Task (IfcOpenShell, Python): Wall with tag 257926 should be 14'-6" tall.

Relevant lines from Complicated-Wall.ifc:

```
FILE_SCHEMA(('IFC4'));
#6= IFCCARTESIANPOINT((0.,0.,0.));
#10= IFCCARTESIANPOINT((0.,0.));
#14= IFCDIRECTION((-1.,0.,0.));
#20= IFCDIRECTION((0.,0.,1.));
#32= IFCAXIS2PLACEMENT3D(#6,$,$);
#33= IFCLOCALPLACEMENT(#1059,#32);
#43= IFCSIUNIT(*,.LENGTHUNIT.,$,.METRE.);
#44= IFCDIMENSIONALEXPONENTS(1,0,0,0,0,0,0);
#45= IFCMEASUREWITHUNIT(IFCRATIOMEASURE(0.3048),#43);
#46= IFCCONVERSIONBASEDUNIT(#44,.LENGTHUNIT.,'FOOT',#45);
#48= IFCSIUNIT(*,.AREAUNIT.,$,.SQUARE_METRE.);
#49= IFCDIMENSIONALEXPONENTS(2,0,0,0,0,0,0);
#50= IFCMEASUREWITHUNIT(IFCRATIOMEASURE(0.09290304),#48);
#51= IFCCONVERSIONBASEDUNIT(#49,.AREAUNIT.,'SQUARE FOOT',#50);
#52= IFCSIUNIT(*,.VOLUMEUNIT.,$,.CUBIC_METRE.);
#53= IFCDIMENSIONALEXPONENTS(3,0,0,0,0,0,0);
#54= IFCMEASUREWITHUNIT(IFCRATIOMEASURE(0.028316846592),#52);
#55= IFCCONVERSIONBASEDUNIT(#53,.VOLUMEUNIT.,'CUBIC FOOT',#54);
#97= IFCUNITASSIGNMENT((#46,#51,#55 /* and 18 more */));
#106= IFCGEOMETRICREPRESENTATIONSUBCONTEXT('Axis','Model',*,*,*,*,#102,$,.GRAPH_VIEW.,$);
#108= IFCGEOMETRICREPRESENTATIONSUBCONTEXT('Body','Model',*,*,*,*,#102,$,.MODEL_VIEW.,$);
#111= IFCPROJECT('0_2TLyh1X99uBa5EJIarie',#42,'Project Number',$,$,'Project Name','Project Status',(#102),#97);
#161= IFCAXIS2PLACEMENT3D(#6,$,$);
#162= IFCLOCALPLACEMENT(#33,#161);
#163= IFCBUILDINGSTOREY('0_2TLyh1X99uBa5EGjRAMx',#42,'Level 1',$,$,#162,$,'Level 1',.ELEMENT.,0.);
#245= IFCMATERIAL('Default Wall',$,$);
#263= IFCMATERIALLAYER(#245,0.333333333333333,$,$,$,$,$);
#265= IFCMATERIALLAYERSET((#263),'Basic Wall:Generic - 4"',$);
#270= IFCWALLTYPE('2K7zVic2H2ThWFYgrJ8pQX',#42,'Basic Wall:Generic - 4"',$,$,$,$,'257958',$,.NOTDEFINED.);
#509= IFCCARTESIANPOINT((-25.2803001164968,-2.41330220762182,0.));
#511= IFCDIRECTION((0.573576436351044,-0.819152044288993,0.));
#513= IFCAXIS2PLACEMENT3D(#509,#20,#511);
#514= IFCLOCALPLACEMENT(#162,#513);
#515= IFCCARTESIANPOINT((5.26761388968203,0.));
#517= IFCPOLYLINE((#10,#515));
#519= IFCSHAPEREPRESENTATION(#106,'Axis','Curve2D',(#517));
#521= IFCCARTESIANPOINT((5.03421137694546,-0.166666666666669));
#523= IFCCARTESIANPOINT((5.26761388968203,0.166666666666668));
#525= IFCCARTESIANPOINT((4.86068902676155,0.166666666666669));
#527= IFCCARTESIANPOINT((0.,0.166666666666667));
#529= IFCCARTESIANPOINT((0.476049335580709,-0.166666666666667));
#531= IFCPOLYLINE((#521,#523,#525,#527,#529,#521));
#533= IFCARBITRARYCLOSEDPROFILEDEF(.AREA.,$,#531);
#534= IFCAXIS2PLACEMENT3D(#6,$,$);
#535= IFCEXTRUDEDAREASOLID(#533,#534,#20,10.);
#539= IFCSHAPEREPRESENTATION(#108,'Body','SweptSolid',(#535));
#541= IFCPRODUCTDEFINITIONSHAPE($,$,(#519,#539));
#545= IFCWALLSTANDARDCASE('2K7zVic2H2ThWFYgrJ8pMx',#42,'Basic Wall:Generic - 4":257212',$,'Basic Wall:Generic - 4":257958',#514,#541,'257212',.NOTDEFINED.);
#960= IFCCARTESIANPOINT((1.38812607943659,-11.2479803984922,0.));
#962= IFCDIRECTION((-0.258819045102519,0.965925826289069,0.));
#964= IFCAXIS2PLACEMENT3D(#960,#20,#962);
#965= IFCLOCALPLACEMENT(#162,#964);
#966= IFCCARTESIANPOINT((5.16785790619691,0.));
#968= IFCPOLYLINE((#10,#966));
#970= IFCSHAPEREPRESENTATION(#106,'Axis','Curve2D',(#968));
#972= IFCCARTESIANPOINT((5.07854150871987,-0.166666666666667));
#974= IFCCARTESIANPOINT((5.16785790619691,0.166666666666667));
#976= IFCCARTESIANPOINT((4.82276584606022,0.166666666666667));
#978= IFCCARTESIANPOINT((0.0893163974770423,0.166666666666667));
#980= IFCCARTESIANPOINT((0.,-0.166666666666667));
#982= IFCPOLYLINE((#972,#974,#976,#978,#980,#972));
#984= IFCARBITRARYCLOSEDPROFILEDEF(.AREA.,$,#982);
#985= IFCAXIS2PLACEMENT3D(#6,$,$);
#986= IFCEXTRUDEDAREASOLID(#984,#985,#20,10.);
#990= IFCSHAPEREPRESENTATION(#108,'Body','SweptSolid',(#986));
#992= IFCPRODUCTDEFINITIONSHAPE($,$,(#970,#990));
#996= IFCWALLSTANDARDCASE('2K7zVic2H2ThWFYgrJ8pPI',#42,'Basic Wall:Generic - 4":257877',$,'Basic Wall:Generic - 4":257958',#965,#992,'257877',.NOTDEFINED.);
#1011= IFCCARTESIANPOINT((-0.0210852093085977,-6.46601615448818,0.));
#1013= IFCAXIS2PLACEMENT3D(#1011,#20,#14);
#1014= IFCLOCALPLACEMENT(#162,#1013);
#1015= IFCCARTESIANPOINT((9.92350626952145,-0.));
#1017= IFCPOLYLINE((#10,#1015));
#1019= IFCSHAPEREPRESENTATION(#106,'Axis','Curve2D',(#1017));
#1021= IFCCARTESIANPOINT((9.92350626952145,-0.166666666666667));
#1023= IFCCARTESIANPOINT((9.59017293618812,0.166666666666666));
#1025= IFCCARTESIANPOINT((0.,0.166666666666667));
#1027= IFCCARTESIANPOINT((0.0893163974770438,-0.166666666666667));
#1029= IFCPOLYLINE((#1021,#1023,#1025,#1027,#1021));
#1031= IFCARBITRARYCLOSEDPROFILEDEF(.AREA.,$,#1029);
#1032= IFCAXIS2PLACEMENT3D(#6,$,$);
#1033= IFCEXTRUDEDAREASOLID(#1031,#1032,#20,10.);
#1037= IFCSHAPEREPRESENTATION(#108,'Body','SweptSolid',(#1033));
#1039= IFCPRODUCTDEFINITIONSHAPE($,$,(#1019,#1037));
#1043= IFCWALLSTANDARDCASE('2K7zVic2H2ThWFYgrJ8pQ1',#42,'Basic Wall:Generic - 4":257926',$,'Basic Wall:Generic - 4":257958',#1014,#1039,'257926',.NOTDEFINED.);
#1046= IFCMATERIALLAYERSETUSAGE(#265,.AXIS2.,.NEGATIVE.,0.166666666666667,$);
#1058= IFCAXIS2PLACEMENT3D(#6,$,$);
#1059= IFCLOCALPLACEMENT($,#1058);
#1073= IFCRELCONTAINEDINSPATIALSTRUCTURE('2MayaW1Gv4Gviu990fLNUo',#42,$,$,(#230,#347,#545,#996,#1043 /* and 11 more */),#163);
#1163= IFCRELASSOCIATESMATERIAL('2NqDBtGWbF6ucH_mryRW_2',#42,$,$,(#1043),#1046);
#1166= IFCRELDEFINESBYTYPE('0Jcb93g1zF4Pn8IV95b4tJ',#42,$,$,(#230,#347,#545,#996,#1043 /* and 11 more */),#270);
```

```python
import ifcopenshell
import ifcopenshell.geom
import ifcopenshell.util.representation
import ifcopenshell.util.shape
import ifcopenshell.util.unit

model = ifcopenshell.open("Complicated-Wall.ifc")
unit_scale = ifcopenshell.util.unit.calculate_unit_scale(model)
settings = ifcopenshell.geom.settings()


def volume(element):
    """Net volume in cubic metres, openings subtracted."""
    shape = ifcopenshell.geom.create_shape(settings, element)
    return ifcopenshell.util.shape.get_volume(shape.geometry)


wall = model.by_guid("2K7zVic2H2ThWFYgrJ8pQ1")
before = volume(wall)

body = ifcopenshell.util.representation.get_representation(wall, "Model", "Body")
solid = body.Items[0]
old_height = solid.Depth
solid.Depth = 174 * 0.0254 / unit_scale
after = volume(wall)

print(f"height {old_height:g} -> {solid.Depth:g}, volume {before:.3f} -> {after:.3f} m3")

model.write("Complicated-Wall_rev.ifc")
```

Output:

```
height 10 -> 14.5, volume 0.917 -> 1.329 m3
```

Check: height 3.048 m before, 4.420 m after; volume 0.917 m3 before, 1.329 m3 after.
